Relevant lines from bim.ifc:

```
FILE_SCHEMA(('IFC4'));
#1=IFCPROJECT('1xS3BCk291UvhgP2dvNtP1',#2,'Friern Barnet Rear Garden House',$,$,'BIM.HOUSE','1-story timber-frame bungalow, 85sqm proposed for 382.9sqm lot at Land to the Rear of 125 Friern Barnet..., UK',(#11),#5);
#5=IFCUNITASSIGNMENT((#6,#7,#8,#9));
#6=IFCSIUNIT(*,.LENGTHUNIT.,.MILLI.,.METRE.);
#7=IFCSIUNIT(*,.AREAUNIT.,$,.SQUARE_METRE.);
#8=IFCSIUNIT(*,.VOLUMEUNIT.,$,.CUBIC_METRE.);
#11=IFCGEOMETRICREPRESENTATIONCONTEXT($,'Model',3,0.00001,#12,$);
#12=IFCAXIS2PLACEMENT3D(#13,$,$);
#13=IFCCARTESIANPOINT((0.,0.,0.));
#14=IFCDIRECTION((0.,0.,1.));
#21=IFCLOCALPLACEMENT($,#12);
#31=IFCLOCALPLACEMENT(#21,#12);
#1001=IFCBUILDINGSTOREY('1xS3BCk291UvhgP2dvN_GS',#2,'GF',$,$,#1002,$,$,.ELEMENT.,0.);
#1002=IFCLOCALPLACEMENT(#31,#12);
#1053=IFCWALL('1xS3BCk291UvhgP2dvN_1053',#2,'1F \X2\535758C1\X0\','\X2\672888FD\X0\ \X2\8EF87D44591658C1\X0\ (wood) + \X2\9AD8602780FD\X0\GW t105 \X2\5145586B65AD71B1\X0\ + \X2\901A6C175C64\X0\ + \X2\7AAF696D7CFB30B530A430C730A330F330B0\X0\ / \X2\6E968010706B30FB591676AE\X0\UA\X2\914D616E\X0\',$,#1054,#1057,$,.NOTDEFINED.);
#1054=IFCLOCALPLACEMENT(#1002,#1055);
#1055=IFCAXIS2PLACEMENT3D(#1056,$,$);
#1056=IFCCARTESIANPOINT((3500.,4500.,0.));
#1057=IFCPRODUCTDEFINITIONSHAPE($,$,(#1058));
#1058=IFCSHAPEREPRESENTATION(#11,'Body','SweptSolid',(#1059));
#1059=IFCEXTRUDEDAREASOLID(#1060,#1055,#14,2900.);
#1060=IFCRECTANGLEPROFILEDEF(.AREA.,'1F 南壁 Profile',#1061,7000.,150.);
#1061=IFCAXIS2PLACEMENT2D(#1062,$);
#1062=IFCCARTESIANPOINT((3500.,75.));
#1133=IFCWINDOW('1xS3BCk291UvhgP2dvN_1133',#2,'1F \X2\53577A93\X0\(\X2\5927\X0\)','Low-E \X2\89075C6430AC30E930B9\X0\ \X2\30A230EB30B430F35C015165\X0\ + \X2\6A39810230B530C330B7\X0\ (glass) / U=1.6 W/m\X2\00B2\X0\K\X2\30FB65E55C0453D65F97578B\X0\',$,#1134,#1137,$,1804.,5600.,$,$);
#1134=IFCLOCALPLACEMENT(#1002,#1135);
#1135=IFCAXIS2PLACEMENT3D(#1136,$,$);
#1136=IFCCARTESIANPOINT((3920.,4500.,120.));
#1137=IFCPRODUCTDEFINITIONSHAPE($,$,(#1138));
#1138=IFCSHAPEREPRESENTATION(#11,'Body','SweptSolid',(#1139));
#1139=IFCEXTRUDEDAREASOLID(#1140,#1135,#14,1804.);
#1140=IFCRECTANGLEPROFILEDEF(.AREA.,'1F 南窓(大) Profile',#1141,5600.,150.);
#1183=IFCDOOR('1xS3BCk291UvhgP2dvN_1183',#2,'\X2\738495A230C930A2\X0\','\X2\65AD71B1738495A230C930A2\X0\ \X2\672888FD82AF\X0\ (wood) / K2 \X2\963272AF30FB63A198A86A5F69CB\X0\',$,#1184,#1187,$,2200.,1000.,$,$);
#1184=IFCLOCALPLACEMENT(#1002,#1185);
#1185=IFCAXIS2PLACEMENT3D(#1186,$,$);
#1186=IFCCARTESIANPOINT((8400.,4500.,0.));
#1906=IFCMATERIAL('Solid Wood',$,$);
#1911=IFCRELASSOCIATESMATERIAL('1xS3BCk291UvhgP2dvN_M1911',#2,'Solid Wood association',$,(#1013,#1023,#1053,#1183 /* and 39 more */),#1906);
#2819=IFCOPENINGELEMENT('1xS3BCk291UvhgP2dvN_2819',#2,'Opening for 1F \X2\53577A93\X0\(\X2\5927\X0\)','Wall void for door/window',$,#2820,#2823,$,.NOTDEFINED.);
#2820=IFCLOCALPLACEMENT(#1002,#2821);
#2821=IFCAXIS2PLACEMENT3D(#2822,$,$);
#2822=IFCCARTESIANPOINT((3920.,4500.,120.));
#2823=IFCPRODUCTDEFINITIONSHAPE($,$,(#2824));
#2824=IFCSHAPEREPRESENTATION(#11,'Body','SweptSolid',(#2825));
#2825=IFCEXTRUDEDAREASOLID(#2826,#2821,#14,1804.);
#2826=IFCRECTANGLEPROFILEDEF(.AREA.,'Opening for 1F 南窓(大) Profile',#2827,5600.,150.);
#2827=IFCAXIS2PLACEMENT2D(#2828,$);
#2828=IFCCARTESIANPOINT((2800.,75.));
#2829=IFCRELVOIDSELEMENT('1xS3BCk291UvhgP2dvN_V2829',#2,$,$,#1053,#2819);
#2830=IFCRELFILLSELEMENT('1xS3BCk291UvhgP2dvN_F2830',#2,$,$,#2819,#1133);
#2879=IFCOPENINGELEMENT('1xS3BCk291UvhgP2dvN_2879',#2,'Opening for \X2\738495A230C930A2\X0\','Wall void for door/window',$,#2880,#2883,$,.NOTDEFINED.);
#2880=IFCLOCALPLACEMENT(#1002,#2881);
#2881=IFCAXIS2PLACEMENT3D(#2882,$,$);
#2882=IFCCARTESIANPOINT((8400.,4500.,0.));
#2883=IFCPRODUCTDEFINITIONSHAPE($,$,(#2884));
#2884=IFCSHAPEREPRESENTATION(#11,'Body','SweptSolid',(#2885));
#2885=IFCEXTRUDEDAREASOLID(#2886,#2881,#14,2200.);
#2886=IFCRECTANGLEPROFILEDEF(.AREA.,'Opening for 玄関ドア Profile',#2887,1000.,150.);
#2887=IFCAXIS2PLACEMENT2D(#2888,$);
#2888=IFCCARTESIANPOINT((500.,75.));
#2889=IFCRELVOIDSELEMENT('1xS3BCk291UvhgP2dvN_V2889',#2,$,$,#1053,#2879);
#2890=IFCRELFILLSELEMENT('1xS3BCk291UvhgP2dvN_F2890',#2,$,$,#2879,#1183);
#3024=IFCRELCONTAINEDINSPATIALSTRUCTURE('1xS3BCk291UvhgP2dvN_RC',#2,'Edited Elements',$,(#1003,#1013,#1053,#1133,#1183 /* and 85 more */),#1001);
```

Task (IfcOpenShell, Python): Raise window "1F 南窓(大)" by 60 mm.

```python
import numpy as np
import ifcopenshell
import ifcopenshell.api.geometry
import ifcopenshell.util.placement
import ifcopenshell.util.unit

model = ifcopenshell.open("bim.ifc")
unit_scale = ifcopenshell.util.unit.calculate_unit_scale(model)

window = model.by_guid("1xS3BCk291UvhgP2dvN_1133")
opening = window.FillsVoids[0].RelatingOpeningElement
dz = 0.06 / unit_scale

shift = np.array([0.0, 0.0, dz])
# The window is not placed relative to its opening, so move both.
for product in (opening, window):
    matrix = ifcopenshell.util.placement.get_local_placement(product.ObjectPlacement)
    matrix[:3, 3] += shift
    ifcopenshell.api.geometry.edit_object_placement(model, product=product, matrix=matrix, is_si=False)

print(f"moved by {dz * unit_scale:+.3f} m")

model.write("bim_rev.ifc")
```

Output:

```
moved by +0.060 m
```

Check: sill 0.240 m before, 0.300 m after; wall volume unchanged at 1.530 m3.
